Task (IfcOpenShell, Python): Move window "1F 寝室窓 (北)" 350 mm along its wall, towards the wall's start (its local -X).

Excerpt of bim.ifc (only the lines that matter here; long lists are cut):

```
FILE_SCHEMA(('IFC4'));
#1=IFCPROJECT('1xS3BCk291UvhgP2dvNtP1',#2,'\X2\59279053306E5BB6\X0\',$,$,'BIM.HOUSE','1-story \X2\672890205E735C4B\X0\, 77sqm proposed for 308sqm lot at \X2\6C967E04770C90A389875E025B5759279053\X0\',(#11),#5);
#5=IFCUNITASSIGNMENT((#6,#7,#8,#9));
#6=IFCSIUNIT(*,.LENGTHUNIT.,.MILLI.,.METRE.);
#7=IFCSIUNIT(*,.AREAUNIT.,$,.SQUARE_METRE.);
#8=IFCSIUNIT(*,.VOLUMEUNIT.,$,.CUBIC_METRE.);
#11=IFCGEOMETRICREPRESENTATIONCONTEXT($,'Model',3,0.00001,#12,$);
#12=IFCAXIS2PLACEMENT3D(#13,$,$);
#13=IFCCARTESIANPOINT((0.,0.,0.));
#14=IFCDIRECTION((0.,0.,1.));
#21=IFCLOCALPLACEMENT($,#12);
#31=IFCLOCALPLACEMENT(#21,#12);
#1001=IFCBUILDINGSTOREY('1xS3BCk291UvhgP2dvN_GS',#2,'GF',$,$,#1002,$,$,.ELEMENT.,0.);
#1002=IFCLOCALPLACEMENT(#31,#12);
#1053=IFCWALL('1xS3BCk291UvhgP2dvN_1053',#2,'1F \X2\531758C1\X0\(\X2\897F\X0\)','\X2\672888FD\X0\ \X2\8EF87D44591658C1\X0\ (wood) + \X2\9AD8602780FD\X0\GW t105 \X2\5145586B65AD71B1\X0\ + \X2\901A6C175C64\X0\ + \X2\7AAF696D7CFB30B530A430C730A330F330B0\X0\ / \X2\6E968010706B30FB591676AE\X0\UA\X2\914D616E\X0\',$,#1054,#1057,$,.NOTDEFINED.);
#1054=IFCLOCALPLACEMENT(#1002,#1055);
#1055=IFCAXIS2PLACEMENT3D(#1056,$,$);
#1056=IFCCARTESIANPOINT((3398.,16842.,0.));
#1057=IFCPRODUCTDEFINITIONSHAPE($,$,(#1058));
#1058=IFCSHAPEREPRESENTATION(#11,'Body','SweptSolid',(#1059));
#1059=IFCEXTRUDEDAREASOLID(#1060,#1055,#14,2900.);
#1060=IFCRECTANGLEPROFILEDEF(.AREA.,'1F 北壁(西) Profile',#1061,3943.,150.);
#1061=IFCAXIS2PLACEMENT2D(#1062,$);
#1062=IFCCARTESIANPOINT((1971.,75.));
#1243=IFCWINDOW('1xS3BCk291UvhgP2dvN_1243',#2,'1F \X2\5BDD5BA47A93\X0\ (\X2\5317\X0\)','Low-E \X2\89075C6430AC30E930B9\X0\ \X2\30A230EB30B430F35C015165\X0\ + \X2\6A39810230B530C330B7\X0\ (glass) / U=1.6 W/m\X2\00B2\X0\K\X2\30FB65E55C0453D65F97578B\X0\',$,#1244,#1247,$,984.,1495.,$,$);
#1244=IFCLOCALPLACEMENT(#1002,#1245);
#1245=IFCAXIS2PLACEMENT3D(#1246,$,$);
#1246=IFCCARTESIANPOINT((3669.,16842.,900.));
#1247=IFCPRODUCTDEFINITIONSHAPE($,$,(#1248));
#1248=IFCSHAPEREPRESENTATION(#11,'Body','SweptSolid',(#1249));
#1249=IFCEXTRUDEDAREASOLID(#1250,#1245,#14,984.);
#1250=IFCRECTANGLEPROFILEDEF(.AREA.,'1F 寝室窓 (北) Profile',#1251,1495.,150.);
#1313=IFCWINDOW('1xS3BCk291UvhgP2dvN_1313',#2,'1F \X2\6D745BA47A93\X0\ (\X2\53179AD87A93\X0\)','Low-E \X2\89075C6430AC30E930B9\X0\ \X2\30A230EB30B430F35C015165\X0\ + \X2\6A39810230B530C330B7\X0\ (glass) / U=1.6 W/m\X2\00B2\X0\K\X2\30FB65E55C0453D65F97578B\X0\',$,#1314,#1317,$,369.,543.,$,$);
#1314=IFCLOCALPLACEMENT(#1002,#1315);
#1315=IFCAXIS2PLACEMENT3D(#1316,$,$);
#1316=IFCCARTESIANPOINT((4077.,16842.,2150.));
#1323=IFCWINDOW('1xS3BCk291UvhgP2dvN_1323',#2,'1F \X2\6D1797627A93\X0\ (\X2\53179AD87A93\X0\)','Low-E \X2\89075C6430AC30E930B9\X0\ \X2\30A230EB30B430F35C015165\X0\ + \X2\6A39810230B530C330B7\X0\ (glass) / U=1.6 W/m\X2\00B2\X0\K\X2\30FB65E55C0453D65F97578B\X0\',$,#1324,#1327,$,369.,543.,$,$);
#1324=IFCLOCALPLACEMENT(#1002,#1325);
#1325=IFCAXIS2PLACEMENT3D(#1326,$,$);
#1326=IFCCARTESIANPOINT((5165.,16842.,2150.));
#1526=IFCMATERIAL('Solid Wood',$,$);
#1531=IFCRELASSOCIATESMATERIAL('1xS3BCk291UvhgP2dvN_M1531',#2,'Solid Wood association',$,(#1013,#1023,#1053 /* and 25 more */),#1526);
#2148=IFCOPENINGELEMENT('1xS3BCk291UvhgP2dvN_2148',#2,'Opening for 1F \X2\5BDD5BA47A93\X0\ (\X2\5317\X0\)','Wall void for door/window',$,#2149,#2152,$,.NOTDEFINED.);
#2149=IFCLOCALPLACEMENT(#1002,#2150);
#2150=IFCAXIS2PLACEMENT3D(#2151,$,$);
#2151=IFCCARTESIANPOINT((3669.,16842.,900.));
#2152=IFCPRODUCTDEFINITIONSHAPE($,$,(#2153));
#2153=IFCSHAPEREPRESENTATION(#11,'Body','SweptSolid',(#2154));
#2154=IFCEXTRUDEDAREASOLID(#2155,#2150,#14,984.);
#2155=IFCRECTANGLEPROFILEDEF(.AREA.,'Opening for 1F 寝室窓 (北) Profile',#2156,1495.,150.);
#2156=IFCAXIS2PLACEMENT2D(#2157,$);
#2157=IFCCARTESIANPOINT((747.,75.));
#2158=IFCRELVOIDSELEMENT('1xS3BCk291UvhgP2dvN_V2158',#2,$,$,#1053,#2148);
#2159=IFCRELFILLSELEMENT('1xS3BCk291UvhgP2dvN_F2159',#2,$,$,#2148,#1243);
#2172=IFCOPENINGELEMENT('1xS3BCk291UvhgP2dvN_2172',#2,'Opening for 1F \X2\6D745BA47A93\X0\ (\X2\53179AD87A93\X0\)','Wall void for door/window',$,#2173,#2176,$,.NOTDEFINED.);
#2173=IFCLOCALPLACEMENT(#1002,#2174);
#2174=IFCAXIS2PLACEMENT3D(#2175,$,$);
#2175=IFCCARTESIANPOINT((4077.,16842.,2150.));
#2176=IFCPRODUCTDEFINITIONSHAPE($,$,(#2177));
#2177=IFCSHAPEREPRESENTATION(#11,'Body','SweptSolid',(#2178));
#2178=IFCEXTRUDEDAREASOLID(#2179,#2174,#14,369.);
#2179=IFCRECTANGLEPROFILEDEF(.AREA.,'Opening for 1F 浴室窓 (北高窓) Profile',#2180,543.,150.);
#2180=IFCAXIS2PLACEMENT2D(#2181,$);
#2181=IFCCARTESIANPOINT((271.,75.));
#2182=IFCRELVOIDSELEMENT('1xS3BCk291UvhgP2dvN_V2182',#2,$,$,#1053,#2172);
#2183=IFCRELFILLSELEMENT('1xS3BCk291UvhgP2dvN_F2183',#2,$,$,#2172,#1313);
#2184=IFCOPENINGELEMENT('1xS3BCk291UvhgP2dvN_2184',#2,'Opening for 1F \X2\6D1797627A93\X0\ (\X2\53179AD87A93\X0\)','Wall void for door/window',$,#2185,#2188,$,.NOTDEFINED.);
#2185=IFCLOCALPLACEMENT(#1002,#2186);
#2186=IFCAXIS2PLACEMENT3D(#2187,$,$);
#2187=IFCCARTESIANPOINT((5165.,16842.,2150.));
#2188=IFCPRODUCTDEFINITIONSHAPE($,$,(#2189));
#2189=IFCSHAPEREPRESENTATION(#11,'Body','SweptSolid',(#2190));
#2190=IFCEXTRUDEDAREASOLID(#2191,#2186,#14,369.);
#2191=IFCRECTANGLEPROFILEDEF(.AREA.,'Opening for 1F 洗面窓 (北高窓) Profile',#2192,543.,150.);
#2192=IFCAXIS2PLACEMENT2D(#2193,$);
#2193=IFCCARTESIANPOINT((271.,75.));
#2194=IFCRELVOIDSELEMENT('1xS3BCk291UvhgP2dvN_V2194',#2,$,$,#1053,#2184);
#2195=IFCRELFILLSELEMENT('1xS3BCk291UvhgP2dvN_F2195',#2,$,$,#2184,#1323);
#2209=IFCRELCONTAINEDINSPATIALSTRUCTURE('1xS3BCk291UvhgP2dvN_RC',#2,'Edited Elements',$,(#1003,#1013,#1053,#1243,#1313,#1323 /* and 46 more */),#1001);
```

```python
import ifcopenshell
import ifcopenshell.api.geometry
import ifcopenshell.util.placement
import ifcopenshell.util.unit

model = ifcopenshell.open("bim.ifc")
unit_scale = ifcopenshell.util.unit.calculate_unit_scale(model)

window = model.by_guid("1xS3BCk291UvhgP2dvN_1243")
opening = window.FillsVoids[0].RelatingOpeningElement
wall = opening.VoidsElements[0].RelatingBuildingElement

wall_matrix = ifcopenshell.util.placement.get_local_placement(wall.ObjectPlacement)
shift = wall_matrix[:3, 0] * -0.35 / unit_scale
before = ifcopenshell.util.placement.get_local_placement(window.ObjectPlacement)[:3, 3].copy()

# The window is not placed relative to its opening, so move both.
for product in (opening, window):
    matrix = ifcopenshell.util.placement.get_local_placement(product.ObjectPlacement)
    matrix[:3, 3] += shift
    ifcopenshell.api.geometry.edit_object_placement(model, product=product, matrix=matrix, is_si=False)

after = ifcopenshell.util.placement.get_local_placement(window.ObjectPlacement)[:3, 3]
print("window moved by", (after - before).round(3) + 0.0)

model.write("bim-out.ifc")
```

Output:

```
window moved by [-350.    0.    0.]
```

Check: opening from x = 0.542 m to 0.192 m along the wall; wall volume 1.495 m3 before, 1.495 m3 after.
